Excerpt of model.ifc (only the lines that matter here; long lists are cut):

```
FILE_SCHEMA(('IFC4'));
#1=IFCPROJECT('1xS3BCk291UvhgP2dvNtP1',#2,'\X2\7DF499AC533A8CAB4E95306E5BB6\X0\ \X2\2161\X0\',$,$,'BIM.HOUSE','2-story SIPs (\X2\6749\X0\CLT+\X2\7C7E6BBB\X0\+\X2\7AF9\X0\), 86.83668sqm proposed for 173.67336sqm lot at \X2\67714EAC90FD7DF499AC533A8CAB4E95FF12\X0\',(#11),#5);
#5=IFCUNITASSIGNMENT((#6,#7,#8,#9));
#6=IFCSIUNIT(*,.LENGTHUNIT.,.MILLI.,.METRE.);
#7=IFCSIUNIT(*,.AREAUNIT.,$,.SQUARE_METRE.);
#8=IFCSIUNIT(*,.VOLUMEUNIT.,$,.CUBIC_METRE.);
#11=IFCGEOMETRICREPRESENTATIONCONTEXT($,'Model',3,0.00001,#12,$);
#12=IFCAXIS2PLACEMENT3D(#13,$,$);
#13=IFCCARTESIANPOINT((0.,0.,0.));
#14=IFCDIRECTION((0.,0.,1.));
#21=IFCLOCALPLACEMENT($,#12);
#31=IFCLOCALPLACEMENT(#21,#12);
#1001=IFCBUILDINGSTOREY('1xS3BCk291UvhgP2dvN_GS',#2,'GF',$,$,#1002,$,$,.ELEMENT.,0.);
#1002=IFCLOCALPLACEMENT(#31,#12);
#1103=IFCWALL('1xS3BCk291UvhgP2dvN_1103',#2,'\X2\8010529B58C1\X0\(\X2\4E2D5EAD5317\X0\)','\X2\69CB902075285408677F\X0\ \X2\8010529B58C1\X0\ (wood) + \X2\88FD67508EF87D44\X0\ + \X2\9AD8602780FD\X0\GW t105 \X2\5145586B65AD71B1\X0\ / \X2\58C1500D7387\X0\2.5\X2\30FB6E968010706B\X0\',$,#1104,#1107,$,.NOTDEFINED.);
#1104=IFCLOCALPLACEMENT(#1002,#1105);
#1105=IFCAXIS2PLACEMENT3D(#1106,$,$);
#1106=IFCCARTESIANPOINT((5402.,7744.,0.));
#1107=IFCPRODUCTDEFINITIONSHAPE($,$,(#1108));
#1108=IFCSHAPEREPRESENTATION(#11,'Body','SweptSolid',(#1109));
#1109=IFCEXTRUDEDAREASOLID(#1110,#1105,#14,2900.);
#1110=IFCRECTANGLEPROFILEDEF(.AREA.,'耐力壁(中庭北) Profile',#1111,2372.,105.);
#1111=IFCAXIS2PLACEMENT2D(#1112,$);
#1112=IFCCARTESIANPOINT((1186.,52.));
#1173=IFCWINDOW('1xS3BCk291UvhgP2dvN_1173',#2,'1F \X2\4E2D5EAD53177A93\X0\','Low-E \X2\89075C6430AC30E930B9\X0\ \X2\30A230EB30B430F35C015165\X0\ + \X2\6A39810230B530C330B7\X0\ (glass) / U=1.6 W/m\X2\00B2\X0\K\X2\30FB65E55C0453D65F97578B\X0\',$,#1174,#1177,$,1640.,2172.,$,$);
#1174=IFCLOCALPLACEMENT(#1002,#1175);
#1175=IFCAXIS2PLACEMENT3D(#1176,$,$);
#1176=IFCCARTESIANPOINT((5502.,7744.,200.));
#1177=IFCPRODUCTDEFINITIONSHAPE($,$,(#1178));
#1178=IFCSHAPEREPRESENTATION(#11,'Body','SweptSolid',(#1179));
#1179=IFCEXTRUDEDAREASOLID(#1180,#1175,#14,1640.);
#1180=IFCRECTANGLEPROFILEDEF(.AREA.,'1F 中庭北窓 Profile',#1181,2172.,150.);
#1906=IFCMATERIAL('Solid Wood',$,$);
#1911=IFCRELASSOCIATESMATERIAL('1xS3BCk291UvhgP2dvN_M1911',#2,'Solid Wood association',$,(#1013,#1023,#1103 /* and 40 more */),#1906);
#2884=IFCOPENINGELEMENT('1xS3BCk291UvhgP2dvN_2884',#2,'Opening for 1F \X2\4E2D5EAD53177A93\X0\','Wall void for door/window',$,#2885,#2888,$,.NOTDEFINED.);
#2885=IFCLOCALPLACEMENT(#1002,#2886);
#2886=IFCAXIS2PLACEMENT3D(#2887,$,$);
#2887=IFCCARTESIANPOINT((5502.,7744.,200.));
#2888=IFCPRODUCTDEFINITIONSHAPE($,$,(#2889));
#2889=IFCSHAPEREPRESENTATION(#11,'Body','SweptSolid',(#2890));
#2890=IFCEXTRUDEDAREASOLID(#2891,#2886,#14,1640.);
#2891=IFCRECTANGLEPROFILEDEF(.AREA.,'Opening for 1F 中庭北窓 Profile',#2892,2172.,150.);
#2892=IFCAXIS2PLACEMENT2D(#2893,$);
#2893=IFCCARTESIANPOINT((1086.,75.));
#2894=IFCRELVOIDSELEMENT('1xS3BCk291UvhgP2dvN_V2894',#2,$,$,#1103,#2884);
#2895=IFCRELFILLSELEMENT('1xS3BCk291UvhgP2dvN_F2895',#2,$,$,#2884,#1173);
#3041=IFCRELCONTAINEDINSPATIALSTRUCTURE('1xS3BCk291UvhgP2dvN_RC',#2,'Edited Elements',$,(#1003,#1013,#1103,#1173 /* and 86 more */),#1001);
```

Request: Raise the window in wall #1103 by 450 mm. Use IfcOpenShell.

```python
import numpy as np
import ifcopenshell
import ifcopenshell.api.geometry
import ifcopenshell.util.placement
import ifcopenshell.util.unit

model = ifcopenshell.open("model.ifc")
unit_scale = ifcopenshell.util.unit.calculate_unit_scale(model)

window = model.by_guid("1xS3BCk291UvhgP2dvN_1173")
opening = window.FillsVoids[0].RelatingOpeningElement
dz = 450.0

shift = np.array([0.0, 0.0, dz])
# The window is not placed relative to its opening, so move both.
for product in (opening, window):
    matrix = ifcopenshell.util.placement.get_local_placement(product.ObjectPlacement)
    matrix[:3, 3] += shift
    ifcopenshell.api.geometry.edit_object_placement(model, product=product, matrix=matrix, is_si=False)

print(f"moved by {dz * unit_scale:+.3f} m")

model.write("model_v2.ifc")
```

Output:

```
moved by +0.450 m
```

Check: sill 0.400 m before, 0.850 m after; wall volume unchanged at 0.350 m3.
